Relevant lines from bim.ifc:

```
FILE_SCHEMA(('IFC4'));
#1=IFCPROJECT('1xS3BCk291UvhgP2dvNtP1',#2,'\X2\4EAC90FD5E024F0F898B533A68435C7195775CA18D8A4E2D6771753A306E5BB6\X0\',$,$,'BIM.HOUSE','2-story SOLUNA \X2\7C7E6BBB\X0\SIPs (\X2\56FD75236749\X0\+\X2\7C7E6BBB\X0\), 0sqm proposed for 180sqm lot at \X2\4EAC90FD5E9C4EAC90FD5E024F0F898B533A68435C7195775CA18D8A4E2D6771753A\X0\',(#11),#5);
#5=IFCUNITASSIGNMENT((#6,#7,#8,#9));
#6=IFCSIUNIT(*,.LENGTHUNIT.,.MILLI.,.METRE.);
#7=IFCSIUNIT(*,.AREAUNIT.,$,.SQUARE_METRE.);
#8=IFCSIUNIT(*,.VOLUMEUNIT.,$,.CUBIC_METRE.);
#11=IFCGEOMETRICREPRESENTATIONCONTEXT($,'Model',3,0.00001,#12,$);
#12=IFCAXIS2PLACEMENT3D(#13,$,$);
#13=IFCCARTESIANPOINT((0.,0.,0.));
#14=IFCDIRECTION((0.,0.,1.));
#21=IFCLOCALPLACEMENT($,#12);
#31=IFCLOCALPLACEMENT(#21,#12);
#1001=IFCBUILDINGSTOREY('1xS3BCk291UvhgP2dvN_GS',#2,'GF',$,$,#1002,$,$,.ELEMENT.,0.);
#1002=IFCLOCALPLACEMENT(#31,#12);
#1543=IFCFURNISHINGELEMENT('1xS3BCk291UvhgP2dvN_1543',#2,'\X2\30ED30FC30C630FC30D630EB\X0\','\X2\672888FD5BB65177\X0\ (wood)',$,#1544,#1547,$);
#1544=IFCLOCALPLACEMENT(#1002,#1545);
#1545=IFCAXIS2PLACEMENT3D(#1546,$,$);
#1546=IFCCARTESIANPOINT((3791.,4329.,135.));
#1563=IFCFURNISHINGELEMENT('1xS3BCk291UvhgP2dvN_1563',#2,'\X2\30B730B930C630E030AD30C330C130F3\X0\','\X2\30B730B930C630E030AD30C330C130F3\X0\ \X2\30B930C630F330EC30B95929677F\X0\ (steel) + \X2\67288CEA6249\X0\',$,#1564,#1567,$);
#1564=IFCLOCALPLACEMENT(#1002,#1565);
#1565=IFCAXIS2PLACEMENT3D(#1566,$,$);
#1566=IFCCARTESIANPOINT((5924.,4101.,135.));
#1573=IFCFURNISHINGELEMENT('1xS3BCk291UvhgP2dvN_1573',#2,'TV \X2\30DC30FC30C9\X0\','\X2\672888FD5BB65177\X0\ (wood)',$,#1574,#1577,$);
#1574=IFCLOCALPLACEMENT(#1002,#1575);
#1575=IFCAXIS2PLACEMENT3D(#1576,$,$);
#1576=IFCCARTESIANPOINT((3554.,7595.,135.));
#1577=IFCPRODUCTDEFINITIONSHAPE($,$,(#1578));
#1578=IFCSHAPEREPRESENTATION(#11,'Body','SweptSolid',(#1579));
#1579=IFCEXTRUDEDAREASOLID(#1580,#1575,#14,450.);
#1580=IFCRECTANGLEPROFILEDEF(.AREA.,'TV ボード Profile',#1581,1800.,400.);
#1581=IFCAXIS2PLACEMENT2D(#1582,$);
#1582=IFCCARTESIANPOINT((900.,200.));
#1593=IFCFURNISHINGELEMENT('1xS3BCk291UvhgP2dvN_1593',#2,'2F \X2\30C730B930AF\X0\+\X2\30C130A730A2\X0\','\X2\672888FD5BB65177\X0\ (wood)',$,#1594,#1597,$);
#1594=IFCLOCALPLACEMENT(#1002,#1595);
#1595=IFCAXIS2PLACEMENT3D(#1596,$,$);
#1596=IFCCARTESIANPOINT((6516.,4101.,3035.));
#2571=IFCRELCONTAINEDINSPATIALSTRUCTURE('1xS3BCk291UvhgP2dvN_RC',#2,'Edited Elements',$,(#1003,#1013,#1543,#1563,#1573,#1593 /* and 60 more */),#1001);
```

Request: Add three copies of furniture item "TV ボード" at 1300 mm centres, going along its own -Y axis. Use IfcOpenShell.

```python
import ifcopenshell
import ifcopenshell.api.geometry
import ifcopenshell.api.root
import ifcopenshell.util.element
import ifcopenshell.util.placement
import ifcopenshell.util.unit

model = ifcopenshell.open("bim.ifc")
unit_scale = ifcopenshell.util.unit.calculate_unit_scale(model)


def reuse_history(source, copy):
    """copy_class also copies each property set's owner history, people and application; keep the originals."""
    for rel in copy.IsDefinedBy:
        if rel.is_a("IfcRelDefinesByProperties") and (history := rel.RelatingPropertyDefinition.OwnerHistory):
            rel.RelatingPropertyDefinition.OwnerHistory = source.OwnerHistory
            ifcopenshell.util.element.remove_deep2(model, history)


source = model.by_guid("1xS3BCk291UvhgP2dvN_1573")
base = ifcopenshell.util.placement.get_local_placement(source.ObjectPlacement)
step = -base[:3, 1] * 1.3 / unit_scale

for i in range(1, 4):
    copy = ifcopenshell.api.root.copy_class(model, product=source)
    copy.Representation = ifcopenshell.util.element.copy_deep(
        model, source.Representation, exclude=["IfcGeometricRepresentationContext", "IfcRepresentationMap"]
    )
    reuse_history(source, copy)
    matrix = base.copy()
    matrix[:3, 3] += i * step
    print("added at", matrix[:3, 3].round(3) + 0.0)
    ifcopenshell.api.geometry.edit_object_placement(model, product=copy, matrix=matrix, is_si=False)

model.write("bim-out.ifc")
```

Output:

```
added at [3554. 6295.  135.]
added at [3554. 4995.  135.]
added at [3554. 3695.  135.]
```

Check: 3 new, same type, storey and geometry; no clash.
